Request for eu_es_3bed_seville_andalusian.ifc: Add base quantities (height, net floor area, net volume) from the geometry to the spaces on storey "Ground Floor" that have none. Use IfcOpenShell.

First a look at what the model holds.

```python
import ifcopenshell
import ifcopenshell.util.element
import ifcopenshell.util.unit

model = ifcopenshell.open("eu_es_3bed_seville_andalusian.ifc")
print(model.schema)
for unit_type in ("LENGTHUNIT", "AREAUNIT", "VOLUMEUNIT"):
    print(unit_type, ifcopenshell.util.unit.calculate_unit_scale(model, unit_type))
storey = next(s for s in model.by_type("IfcBuildingStorey") if s.Name == "Ground Floor")
spaces = [e for e in ifcopenshell.util.element.get_decomposition(storey) if e.is_a("IfcSpace")]
for e in sorted(spaces, key=lambda e: e.id()):
    print(e.id(), e.is_a(), e.Name, list(ifcopenshell.util.element.get_psets(e, qtos_only=True)), sep=" | ")
```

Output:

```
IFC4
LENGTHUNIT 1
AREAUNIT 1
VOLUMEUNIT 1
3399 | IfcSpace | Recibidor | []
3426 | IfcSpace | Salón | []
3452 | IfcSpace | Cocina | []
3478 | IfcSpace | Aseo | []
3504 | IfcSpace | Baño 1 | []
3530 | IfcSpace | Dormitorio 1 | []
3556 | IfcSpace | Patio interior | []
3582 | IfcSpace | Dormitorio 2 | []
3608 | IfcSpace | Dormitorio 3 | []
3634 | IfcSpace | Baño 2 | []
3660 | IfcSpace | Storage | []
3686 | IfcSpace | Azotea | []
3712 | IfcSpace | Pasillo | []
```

```python
import ifcopenshell
import ifcopenshell.api.pset
import ifcopenshell.geom
import ifcopenshell.util.element
import ifcopenshell.util.shape
import ifcopenshell.util.unit

model = ifcopenshell.open("eu_es_3bed_seville_andalusian.ifc")
unit_scale = ifcopenshell.util.unit.calculate_unit_scale(model)
area_scale = ifcopenshell.util.unit.calculate_unit_scale(model, "AREAUNIT")
volume_scale = ifcopenshell.util.unit.calculate_unit_scale(model, "VOLUMEUNIT")
settings = ifcopenshell.geom.settings()

storey = next(s for s in model.by_type("IfcBuildingStorey") if s.Name == "Ground Floor")
spaces = [e for e in ifcopenshell.util.element.get_decomposition(storey) if e.is_a("IfcSpace")]

for e in sorted(spaces, key=lambda e: e.id()):
    if ifcopenshell.util.element.get_psets(e, qtos_only=True, should_inherit=False):
        continue
    # Geometry comes back in metres, in the element's own axes.
    shape = ifcopenshell.geom.create_shape(settings, e)
    values = {
        "Height": ifcopenshell.util.shape.get_z(shape.geometry) / unit_scale,
        "NetFloorArea": ifcopenshell.util.shape.get_footprint_area(shape.geometry) / area_scale,
        "NetVolume": ifcopenshell.util.shape.get_volume(shape.geometry) / volume_scale,
    }
    qto = ifcopenshell.api.pset.add_qto(model, product=e, name="Qto_SpaceBaseQuantities")
    ifcopenshell.api.pset.edit_qto(model, qto=qto, properties=values)
    print(e.id(), {k: round(v, 3) for k, v in values.items()})

model.write("eu_es_3bed_seville_andalusian_edited.ifc")
```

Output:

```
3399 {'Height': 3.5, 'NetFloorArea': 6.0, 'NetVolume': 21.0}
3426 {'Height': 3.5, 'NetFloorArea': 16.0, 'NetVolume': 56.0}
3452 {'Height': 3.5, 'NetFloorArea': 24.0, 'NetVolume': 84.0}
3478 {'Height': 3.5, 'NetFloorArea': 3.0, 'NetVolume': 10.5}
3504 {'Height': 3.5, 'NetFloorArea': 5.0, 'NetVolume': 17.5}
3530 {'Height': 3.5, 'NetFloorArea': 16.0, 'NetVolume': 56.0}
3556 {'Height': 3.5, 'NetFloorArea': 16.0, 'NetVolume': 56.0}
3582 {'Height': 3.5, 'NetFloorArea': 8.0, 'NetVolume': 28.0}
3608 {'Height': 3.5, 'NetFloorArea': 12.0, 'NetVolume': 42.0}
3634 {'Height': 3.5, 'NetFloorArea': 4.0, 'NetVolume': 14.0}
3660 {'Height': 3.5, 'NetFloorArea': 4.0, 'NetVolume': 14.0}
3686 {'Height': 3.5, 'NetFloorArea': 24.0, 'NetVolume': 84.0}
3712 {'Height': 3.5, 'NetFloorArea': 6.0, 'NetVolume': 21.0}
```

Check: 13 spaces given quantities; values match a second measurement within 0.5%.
